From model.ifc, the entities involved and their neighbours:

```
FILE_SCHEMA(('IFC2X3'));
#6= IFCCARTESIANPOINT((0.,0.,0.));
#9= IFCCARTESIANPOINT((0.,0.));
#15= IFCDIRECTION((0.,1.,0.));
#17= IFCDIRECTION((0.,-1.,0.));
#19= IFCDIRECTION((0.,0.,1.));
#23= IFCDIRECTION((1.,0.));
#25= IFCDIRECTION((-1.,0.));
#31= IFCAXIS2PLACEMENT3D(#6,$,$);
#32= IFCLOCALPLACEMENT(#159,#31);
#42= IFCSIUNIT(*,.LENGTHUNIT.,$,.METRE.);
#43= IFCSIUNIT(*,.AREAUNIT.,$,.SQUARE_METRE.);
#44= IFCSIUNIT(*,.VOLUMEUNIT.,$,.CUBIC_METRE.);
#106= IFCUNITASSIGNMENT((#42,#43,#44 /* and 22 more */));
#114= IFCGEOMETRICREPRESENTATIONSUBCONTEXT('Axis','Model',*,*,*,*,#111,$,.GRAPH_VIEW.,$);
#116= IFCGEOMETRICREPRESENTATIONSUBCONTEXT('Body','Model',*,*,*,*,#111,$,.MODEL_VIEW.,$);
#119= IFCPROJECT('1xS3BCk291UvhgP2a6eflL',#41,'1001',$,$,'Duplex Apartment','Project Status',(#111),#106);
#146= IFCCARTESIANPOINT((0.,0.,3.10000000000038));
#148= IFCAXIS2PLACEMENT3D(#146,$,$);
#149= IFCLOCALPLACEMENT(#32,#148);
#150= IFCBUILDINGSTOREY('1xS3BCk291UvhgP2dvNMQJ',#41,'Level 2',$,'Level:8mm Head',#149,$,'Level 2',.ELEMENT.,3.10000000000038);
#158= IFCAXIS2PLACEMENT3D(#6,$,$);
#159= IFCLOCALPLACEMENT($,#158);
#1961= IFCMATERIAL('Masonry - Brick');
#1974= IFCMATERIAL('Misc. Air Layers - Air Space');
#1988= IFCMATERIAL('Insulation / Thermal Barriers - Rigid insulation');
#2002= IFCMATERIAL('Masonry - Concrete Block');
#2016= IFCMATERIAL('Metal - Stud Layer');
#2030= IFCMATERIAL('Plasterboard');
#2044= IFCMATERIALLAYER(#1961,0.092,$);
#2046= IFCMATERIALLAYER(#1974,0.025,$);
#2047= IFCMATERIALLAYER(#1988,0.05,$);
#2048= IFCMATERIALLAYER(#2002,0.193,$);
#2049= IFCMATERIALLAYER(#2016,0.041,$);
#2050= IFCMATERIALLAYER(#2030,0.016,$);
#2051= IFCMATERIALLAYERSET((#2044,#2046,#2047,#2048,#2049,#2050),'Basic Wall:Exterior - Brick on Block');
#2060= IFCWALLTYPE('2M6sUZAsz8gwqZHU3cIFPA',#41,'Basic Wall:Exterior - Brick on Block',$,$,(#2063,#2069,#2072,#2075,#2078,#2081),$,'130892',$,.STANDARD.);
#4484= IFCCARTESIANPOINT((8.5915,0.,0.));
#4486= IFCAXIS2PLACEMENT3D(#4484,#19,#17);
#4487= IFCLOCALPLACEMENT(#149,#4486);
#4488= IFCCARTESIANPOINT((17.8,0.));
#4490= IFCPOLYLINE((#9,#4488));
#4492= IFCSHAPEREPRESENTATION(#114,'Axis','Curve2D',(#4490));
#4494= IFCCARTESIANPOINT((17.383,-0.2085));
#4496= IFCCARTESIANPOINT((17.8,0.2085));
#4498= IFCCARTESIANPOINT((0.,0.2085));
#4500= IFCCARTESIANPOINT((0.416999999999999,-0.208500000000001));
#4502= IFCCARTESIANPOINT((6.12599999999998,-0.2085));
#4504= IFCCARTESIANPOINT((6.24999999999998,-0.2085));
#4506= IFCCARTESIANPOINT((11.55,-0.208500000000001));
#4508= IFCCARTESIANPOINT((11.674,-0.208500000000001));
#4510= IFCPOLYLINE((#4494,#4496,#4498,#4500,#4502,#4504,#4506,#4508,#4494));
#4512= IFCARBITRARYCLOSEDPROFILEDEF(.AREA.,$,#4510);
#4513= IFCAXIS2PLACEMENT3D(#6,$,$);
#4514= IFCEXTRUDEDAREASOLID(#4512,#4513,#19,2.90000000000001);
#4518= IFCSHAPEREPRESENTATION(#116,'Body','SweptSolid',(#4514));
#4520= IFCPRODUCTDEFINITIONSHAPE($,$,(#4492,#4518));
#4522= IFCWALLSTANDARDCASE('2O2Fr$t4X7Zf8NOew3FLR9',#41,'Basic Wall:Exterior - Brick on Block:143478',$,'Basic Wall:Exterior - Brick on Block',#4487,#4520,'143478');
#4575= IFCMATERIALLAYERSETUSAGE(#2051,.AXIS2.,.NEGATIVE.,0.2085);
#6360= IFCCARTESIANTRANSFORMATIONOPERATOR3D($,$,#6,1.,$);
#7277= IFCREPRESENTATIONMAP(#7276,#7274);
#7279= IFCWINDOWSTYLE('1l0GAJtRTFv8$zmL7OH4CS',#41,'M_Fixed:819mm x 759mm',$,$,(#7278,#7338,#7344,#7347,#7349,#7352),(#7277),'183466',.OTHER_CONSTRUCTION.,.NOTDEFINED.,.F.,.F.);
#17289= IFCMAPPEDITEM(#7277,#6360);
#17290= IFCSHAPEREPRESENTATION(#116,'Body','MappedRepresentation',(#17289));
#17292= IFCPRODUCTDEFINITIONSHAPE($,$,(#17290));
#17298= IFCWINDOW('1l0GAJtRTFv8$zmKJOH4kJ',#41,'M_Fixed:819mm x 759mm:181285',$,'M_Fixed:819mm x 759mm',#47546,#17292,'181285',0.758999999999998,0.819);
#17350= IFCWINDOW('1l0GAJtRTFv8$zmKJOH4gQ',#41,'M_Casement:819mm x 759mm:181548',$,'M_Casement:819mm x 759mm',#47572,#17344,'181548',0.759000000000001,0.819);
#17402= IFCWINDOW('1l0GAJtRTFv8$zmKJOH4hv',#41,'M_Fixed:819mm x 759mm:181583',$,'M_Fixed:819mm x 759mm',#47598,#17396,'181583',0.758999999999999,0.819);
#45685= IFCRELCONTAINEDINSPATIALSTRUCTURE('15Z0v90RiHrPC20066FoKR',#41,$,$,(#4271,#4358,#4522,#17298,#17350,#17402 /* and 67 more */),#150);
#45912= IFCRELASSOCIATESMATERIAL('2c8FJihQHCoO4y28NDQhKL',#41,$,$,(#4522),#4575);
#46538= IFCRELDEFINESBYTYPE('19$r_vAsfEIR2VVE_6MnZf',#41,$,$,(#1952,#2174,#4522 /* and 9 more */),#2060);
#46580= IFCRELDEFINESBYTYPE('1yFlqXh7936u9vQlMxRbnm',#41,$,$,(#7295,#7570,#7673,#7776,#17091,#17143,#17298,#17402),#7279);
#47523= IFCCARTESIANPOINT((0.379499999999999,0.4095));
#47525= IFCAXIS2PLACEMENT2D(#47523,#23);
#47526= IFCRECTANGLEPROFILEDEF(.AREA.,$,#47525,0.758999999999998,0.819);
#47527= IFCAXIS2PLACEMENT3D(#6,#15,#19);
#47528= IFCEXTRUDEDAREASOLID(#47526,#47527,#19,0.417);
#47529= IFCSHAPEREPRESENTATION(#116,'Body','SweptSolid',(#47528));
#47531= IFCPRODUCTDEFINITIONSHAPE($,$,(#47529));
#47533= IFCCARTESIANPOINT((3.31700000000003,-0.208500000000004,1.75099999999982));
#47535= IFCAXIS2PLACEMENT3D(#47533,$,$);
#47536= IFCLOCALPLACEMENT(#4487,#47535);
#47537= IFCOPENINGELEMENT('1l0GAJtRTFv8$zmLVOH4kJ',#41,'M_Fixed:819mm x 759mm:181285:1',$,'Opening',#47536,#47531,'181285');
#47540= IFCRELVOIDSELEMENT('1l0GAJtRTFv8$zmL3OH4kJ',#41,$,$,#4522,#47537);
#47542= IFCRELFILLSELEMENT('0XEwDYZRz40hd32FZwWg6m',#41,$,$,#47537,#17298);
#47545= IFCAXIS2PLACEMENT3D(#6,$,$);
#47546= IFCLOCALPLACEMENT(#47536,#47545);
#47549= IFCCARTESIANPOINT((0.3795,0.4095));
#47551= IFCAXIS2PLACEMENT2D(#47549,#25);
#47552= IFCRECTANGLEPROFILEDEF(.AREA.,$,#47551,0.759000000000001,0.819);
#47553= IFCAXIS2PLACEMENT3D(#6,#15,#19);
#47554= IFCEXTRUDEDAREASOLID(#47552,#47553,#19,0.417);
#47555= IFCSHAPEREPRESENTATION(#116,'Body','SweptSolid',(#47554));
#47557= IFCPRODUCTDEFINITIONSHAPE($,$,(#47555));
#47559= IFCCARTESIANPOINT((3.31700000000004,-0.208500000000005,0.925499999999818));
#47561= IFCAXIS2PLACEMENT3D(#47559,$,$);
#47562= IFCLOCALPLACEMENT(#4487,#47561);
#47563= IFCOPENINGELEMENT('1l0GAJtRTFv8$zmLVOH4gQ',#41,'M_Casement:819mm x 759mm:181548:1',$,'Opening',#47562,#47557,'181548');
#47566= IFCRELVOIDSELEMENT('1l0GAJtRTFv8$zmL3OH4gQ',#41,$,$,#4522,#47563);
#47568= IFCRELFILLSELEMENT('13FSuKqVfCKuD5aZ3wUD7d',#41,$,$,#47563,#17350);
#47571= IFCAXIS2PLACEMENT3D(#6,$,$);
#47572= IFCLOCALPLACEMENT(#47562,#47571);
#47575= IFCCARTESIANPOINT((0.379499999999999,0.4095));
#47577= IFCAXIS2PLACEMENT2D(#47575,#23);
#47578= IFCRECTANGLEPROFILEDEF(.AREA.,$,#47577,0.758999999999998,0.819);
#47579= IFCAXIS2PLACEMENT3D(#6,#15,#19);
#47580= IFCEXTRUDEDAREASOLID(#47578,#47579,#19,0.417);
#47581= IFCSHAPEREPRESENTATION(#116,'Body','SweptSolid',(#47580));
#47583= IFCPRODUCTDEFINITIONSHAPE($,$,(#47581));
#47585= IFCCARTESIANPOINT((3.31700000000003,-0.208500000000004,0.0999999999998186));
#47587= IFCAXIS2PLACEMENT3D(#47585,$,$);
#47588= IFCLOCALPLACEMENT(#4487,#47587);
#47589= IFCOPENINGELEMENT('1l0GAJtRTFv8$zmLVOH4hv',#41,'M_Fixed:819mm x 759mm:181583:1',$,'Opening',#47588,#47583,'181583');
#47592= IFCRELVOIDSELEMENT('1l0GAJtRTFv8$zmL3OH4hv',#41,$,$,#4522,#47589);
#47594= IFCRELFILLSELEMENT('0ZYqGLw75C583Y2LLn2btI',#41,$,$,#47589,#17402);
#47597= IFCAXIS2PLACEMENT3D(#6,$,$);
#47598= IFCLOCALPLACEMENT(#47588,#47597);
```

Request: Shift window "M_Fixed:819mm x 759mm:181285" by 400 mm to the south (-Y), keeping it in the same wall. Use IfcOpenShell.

```python
import ifcopenshell
import ifcopenshell.api.geometry
import ifcopenshell.util.placement
import ifcopenshell.util.unit

model = ifcopenshell.open("model.ifc")
unit_scale = ifcopenshell.util.unit.calculate_unit_scale(model)

window = model.by_guid("1l0GAJtRTFv8$zmKJOH4kJ")
opening = window.FillsVoids[0].RelatingOpeningElement
wall = opening.VoidsElements[0].RelatingBuildingElement

wall_matrix = ifcopenshell.util.placement.get_local_placement(wall.ObjectPlacement)
shift = wall_matrix[:3, 0] * 0.4 / unit_scale
before = ifcopenshell.util.placement.get_local_placement(window.ObjectPlacement)[:3, 3].copy()

# The window is placed relative to its opening, so it follows when the opening moves.
matrix = ifcopenshell.util.placement.get_local_placement(opening.ObjectPlacement)
matrix[:3, 3] += shift
ifcopenshell.api.geometry.edit_object_placement(
    model, product=opening, matrix=matrix, is_si=False, should_transform_children=True
)

after = ifcopenshell.util.placement.get_local_placement(window.ObjectPlacement)[:3, 3]
print("window moved by", (after - before).round(3) + 0.0)

model.write("model_updated.ifc")
```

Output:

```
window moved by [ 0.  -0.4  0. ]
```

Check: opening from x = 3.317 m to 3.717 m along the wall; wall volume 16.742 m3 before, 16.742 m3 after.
